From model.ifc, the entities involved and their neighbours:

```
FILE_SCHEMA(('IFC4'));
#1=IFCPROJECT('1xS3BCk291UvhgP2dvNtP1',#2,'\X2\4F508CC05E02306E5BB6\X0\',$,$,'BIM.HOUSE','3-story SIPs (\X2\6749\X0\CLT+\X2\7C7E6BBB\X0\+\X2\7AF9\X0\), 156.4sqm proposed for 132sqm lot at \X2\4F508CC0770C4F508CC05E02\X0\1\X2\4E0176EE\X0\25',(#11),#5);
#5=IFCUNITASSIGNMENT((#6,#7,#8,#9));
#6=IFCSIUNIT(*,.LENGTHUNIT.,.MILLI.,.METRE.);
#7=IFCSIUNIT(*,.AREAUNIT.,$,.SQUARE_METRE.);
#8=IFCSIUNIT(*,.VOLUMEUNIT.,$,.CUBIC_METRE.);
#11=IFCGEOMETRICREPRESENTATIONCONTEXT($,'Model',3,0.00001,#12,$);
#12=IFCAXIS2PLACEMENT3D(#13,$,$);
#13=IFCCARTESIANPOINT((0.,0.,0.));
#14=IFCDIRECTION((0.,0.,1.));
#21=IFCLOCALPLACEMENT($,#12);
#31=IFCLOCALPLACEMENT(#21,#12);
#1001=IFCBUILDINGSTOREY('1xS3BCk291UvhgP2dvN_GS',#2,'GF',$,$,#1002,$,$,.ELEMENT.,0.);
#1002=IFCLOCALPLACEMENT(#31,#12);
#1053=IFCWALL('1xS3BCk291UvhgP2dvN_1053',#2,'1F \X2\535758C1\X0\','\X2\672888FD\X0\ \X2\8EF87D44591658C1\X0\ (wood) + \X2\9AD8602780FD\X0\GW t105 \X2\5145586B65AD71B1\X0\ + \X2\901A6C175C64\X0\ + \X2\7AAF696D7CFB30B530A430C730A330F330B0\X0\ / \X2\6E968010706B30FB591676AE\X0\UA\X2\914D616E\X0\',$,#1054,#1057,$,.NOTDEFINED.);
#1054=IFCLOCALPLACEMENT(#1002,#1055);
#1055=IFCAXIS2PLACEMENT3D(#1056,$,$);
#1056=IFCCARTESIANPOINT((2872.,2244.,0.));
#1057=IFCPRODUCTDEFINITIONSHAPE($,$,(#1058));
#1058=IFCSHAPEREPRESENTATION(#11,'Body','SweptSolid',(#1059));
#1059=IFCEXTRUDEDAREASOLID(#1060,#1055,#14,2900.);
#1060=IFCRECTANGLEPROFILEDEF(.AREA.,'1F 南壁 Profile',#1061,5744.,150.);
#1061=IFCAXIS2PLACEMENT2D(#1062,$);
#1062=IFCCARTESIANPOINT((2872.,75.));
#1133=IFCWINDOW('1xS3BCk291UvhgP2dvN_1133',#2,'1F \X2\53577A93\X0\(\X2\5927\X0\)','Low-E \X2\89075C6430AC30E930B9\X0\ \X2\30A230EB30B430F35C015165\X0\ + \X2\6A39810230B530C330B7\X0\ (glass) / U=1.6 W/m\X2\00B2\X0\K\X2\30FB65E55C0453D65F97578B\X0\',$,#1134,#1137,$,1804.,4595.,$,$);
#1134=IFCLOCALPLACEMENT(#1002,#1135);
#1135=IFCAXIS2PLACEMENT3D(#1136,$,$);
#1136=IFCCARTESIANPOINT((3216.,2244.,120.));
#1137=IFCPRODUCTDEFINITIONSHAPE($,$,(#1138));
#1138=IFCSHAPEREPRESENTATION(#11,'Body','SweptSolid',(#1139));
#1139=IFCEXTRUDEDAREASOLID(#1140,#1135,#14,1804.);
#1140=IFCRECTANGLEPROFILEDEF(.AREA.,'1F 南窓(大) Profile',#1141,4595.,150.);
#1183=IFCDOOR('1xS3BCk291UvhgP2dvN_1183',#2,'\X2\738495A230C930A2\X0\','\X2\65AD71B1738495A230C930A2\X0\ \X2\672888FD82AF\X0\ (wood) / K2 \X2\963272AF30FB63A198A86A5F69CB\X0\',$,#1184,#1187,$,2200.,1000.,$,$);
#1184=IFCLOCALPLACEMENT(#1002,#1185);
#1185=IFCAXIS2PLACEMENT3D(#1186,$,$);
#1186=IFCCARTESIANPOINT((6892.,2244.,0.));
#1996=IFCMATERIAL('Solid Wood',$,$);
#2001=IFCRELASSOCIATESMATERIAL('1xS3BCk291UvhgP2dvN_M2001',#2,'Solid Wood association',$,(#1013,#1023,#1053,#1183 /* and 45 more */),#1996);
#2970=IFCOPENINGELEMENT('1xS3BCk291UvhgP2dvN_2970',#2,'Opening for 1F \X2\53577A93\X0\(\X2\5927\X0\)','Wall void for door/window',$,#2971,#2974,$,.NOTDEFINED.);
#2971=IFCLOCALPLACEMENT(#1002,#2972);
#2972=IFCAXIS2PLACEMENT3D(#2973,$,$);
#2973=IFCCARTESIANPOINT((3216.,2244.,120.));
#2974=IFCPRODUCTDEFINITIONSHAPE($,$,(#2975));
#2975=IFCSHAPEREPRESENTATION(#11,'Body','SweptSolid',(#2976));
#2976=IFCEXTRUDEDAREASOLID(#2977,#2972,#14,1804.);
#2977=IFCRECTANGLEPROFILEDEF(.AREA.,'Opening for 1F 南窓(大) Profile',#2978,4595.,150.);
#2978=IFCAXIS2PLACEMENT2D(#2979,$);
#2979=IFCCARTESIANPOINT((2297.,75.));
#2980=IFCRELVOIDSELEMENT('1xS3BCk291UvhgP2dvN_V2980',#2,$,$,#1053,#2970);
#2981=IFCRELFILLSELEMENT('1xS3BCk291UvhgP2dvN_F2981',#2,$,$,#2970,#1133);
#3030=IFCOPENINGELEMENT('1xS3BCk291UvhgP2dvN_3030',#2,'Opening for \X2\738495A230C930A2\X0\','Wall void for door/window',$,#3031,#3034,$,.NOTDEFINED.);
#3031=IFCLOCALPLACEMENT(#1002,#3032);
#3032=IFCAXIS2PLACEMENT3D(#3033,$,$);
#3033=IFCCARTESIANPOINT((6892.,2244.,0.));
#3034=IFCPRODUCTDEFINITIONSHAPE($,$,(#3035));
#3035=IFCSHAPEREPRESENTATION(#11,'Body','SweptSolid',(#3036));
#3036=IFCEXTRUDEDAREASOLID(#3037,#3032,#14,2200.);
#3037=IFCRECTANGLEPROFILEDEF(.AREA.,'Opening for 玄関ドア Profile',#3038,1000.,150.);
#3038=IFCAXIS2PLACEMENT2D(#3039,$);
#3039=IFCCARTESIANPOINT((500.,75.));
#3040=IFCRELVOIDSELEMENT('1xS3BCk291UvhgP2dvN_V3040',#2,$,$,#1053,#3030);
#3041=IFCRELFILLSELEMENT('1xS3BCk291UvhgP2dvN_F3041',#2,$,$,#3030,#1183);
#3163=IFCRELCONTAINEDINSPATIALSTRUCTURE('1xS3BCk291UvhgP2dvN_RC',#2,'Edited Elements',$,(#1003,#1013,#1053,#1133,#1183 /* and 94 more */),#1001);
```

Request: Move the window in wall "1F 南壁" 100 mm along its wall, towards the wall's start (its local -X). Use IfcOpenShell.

```python
import ifcopenshell
import ifcopenshell.api.geometry
import ifcopenshell.util.placement

model = ifcopenshell.open("model.ifc")

window = model.by_guid("1xS3BCk291UvhgP2dvN_1133")
opening = window.FillsVoids[0].RelatingOpeningElement
wall = opening.VoidsElements[0].RelatingBuildingElement

wall_matrix = ifcopenshell.util.placement.get_local_placement(wall.ObjectPlacement)
shift = wall_matrix[:3, 0] * -100.0
before = ifcopenshell.util.placement.get_local_placement(window.ObjectPlacement)[:3, 3].copy()

# The window is not placed relative to its opening, so move both.
for product in (opening, window):
    matrix = ifcopenshell.util.placement.get_local_placement(product.ObjectPlacement)
    matrix[:3, 3] += shift
    ifcopenshell.api.geometry.edit_object_placement(model, product=product, matrix=matrix, is_si=False)

after = ifcopenshell.util.placement.get_local_placement(window.ObjectPlacement)[:3, 3]
print("window moved by", (after - before).round(3) + 0.0)

model.write("model_updated.ifc")
```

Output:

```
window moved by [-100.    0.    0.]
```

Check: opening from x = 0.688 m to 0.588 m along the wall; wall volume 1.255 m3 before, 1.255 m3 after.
